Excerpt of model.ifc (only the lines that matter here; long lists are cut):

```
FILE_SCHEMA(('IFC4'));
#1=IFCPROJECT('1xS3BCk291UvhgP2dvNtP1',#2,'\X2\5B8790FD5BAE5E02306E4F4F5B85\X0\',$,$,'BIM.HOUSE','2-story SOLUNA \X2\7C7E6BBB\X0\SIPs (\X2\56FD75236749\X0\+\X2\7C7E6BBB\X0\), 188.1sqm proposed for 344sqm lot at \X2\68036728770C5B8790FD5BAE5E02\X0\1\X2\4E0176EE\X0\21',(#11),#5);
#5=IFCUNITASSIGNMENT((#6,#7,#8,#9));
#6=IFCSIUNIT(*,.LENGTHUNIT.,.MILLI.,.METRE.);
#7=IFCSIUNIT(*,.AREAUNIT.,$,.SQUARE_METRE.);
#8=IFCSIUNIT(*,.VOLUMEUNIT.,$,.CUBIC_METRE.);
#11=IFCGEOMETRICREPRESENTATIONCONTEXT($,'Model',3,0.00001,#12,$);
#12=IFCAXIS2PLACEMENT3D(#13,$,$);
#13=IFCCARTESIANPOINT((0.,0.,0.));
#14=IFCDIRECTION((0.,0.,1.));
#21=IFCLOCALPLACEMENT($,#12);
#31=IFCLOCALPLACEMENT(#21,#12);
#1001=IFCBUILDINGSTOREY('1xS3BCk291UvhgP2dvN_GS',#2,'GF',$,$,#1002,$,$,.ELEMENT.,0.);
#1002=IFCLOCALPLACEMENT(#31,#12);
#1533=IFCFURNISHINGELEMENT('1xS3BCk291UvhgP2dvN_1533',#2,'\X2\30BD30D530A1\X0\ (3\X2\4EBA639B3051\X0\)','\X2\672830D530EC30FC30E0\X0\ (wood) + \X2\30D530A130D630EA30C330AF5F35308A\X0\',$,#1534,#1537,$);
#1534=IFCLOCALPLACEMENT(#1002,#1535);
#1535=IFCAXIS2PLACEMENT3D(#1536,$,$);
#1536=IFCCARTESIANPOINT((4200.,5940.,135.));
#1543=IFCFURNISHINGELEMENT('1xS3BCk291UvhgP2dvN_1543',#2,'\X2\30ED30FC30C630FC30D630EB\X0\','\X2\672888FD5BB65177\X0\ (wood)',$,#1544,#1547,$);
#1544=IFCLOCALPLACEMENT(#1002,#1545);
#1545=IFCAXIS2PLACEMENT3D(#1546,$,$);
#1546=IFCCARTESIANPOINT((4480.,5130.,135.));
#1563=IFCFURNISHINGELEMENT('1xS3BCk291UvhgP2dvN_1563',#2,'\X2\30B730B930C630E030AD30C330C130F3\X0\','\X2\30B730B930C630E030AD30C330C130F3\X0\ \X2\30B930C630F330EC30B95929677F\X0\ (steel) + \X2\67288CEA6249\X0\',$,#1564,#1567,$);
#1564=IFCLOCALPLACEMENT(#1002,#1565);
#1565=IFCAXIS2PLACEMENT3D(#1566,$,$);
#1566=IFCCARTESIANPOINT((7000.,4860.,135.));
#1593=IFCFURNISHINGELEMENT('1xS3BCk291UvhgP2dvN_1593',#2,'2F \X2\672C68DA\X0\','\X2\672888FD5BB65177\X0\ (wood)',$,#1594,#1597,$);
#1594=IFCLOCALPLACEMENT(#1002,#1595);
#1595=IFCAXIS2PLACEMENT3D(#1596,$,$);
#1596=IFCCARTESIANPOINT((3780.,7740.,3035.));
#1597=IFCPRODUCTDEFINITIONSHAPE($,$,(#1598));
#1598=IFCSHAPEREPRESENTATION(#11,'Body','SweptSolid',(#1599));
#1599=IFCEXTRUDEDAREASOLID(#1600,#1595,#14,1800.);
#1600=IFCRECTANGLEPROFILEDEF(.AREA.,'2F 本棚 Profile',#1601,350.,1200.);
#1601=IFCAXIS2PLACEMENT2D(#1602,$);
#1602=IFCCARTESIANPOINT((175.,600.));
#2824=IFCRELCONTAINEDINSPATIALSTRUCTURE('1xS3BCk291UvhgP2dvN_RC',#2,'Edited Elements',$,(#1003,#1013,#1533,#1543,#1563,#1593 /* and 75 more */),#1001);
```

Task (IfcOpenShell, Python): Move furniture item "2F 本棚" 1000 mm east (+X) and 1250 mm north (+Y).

```python
import ifcopenshell
import ifcopenshell.api.geometry
import ifcopenshell.util.placement
import ifcopenshell.util.unit

model = ifcopenshell.open("model.ifc")
unit_scale = ifcopenshell.util.unit.calculate_unit_scale(model)

item = model.by_id(1593)
matrix = ifcopenshell.util.placement.get_local_placement(item.ObjectPlacement)
matrix[0, 3] += 1 / unit_scale
matrix[1, 3] += 1.25 / unit_scale
ifcopenshell.api.geometry.edit_object_placement(model, product=item, matrix=matrix, is_si=False)

print(ifcopenshell.util.placement.get_local_placement(item.ObjectPlacement).round(3) + 0.0)

model.write("model_updated.ifc")
```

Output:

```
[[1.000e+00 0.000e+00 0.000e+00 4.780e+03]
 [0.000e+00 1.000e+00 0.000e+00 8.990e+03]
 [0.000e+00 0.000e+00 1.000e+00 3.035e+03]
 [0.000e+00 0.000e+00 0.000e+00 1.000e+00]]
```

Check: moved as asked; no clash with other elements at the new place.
